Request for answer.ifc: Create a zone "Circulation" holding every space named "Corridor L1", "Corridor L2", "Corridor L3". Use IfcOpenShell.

First a look at what the model holds.

```python
import ifcopenshell

model = ifcopenshell.open("answer.ifc")
print(model.schema)
seen = {}
for space in model.by_type("IfcSpace"):
    seen[space.Name] = seen.get(space.Name, 0) + 1
for name, count in sorted(seen.items(), key=str):
    print(count, "x", name)
print("zones:", [z.Name for z in model.by_type("IfcZone")][:20])
```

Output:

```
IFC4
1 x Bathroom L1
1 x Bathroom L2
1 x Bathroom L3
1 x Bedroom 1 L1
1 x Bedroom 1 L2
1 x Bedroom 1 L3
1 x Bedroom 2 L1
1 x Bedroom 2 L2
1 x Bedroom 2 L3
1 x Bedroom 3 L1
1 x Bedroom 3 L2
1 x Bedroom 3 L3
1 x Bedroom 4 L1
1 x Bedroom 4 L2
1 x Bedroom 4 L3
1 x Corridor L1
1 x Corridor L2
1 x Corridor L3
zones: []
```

```python
import ifcopenshell
import ifcopenshell.api.group
import ifcopenshell.api.root

model = ifcopenshell.open("answer.ifc")

names = {"Corridor L1", "Corridor L2", "Corridor L3"}
spaces = [s for s in model.by_type("IfcSpace") if s.Name in names]

zone = ifcopenshell.api.root.create_entity(model, ifc_class="IfcZone", name="Circulation")
ifcopenshell.api.group.assign_group(model, products=spaces, group=zone)
print(len(spaces), "spaces in", zone.Name)

model.write("answer_rev.ifc")
```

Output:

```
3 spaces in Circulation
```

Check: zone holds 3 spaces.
